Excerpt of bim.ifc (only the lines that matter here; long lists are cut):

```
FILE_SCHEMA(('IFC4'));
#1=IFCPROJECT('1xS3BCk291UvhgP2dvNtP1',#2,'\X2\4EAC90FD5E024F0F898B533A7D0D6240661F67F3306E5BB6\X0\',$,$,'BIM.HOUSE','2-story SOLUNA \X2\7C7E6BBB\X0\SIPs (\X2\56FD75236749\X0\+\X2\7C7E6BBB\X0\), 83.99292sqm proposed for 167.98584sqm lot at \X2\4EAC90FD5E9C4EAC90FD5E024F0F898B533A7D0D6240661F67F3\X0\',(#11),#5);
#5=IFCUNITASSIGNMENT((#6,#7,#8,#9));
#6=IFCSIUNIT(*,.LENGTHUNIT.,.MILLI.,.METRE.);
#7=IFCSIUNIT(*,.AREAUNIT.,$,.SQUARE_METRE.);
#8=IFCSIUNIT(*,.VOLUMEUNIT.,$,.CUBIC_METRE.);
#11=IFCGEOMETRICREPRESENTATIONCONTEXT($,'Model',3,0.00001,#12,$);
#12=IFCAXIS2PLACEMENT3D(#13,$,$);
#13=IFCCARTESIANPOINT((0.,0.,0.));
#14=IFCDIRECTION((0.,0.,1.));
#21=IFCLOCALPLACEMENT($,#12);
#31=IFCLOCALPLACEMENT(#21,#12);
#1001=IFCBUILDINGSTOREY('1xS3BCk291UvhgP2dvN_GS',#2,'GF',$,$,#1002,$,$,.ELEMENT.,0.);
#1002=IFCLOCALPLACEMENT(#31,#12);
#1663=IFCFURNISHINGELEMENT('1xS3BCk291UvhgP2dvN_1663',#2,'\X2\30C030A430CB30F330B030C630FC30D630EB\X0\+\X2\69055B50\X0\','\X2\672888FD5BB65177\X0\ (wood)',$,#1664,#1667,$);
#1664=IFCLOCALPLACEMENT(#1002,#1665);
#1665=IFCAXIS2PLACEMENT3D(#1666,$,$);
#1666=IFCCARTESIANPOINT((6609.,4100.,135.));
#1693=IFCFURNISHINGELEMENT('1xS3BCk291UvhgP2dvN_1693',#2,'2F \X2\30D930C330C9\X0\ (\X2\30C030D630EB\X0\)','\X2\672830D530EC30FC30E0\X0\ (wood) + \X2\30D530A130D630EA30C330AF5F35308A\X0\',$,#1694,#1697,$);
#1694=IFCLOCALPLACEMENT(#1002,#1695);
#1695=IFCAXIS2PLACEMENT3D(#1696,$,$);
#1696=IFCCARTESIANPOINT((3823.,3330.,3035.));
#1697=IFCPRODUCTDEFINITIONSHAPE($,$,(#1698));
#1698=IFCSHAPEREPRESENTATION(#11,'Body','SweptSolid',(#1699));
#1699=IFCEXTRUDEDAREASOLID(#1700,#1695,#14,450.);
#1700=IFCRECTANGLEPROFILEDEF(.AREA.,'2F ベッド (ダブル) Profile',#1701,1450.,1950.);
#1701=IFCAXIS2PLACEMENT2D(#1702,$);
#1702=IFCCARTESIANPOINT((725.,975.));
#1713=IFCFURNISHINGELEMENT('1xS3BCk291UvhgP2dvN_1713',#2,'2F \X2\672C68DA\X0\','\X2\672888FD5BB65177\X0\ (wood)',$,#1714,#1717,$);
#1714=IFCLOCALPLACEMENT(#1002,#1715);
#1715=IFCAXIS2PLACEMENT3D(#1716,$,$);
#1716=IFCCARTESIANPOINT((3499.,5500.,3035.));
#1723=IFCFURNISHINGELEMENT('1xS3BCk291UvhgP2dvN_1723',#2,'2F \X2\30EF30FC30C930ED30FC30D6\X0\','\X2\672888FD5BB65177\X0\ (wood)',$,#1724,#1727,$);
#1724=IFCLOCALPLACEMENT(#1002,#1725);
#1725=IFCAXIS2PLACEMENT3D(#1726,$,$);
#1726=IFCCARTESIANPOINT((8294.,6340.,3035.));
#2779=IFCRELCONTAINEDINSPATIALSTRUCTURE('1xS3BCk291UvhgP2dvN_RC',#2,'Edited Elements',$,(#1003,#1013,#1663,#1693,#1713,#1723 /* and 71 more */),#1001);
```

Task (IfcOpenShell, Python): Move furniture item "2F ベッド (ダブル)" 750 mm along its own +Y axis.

```python
import ifcopenshell
import ifcopenshell.api.geometry
import ifcopenshell.util.placement

model = ifcopenshell.open("bim.ifc")

item = model.by_guid("1xS3BCk291UvhgP2dvN_1693")
matrix = ifcopenshell.util.placement.get_local_placement(item.ObjectPlacement)
matrix[:3, 3] += matrix[:3, 1] * 750.0
ifcopenshell.api.geometry.edit_object_placement(model, product=item, matrix=matrix, is_si=False)

print(ifcopenshell.util.placement.get_local_placement(item.ObjectPlacement).round(3) + 0.0)

model.write("bim_edited.ifc")
```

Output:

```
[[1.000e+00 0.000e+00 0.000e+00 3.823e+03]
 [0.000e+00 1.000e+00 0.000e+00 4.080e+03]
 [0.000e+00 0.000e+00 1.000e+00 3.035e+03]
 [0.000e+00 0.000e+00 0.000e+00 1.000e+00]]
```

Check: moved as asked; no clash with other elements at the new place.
